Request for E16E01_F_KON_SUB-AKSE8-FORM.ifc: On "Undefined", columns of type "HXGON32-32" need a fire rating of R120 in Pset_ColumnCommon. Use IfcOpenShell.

First a look at what the model holds.

```python
import ifcopenshell
import ifcopenshell.util.element

model = ifcopenshell.open("E16E01_F_KON_SUB-AKSE8-FORM.ifc")
print(model.schema)
storey = next(s for s in model.by_type("IfcBuildingStorey") if s.Name == "Undefined")
columns = [e for e in ifcopenshell.util.element.get_decomposition(storey) if e.is_a("IfcColumn")]
seen = {}
for e in columns:
    element_type = ifcopenshell.util.element.get_type(e)
    key = (element_type.Name if element_type != e and element_type else None, ifcopenshell.util.element.get_pset(e, "Pset_ColumnCommon", "FireRating"))
    seen[key] = seen.get(key, 0) + 1
for (name, value), count in sorted(seen.items(), key=str):
    print(count, "x", name, "|", value)
```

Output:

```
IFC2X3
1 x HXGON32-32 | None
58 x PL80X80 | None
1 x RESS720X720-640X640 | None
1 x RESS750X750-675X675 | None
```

```python
import ifcopenshell
import ifcopenshell.api.pset
import ifcopenshell.util.element

model = ifcopenshell.open("E16E01_F_KON_SUB-AKSE8-FORM.ifc")

storey = next(s for s in model.by_type("IfcBuildingStorey") if s.Name == "Undefined")
columns = [e for e in ifcopenshell.util.element.get_decomposition(storey) if e.is_a("IfcColumn")]

count = 0
for e in columns:
    element_type = ifcopenshell.util.element.get_type(e)
    if element_type in (None, e) or element_type.Name != "HXGON32-32":
        continue
    # add_pset returns the element's existing set when there is one.
    pset = ifcopenshell.api.pset.add_pset(model, product=e, name="Pset_ColumnCommon")
    ifcopenshell.api.pset.edit_pset(model, pset=pset, properties={"FireRating": "R120"})
    count += 1

print(count, "columns updated")

model.write("E16E01_F_KON_SUB-AKSE8-FORM-out.ifc")
```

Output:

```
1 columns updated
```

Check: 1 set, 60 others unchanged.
